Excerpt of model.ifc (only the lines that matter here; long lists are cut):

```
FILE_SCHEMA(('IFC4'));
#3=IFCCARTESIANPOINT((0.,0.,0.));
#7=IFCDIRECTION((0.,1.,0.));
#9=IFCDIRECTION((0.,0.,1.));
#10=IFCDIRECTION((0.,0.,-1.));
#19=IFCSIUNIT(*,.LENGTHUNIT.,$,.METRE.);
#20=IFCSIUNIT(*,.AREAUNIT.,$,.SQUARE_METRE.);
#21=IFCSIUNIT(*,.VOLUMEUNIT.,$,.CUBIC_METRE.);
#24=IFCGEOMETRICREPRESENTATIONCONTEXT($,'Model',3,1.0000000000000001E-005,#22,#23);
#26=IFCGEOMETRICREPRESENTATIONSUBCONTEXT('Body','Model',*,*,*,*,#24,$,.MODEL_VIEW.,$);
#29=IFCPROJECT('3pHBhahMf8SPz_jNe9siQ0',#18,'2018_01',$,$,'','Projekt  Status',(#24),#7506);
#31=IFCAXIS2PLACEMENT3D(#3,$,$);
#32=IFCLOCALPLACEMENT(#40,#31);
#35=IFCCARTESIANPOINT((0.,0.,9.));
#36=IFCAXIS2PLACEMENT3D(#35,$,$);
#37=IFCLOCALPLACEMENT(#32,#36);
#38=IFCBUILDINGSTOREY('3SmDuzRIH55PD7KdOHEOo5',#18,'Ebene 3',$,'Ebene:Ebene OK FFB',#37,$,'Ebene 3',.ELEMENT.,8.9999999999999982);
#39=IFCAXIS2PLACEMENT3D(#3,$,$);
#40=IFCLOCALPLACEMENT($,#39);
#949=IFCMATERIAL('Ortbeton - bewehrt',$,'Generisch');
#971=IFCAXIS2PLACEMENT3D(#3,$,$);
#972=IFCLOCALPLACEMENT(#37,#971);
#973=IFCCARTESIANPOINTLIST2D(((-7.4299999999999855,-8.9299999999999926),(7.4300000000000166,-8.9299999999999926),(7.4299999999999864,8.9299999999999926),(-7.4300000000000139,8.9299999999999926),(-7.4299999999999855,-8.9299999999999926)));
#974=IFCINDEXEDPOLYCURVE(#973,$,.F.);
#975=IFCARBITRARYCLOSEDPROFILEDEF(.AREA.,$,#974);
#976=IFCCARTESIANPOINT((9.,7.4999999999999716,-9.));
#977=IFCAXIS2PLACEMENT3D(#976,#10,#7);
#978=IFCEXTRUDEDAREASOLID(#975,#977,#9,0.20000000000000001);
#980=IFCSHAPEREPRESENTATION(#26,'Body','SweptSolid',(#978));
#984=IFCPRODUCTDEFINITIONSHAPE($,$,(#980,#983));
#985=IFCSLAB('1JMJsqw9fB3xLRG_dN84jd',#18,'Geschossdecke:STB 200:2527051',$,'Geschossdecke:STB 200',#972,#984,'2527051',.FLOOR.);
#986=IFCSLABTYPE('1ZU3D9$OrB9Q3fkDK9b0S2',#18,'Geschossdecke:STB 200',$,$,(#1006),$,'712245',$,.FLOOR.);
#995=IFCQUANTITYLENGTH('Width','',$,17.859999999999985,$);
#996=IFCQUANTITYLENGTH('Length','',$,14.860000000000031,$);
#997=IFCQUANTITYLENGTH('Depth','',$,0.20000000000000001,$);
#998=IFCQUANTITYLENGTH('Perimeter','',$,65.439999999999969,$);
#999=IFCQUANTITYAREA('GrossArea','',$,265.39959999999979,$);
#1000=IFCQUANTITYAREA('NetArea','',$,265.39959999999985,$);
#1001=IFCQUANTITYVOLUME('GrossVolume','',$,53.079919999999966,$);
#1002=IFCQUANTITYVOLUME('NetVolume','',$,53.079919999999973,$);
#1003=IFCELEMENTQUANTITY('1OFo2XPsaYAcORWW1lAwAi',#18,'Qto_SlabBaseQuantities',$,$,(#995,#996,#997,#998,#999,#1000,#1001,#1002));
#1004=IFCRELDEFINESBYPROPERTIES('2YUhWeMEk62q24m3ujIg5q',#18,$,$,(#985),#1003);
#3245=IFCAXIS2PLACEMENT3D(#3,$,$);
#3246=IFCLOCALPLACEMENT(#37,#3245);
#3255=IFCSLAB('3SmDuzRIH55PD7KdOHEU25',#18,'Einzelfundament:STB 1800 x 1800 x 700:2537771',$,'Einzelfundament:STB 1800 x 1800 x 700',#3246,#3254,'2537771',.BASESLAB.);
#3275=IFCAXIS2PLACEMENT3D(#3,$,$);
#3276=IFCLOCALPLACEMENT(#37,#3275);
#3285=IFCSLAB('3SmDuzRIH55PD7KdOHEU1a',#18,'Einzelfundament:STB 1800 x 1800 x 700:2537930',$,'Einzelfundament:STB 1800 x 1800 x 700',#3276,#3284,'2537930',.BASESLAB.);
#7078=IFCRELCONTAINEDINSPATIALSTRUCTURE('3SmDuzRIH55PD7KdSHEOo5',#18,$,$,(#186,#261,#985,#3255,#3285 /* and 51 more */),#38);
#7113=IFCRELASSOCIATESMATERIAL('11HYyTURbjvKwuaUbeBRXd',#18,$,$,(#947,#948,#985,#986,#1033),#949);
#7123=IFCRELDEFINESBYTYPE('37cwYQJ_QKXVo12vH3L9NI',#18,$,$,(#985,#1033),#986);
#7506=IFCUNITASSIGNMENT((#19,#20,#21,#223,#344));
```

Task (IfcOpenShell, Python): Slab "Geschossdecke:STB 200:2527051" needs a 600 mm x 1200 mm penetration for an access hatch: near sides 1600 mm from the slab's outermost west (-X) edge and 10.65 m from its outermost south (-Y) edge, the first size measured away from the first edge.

```python
import numpy as np
import ifcopenshell
import ifcopenshell.api.feature
import ifcopenshell.api.geometry
import ifcopenshell.api.pset
import ifcopenshell.api.root
import ifcopenshell.geom
import ifcopenshell.util.element
import ifcopenshell.util.placement
import ifcopenshell.util.representation
import ifcopenshell.util.shape
import ifcopenshell.util.unit

model = ifcopenshell.open("model.ifc")
unit_scale = ifcopenshell.util.unit.calculate_unit_scale(model)
area_scale = ifcopenshell.util.unit.calculate_unit_scale(model, "AREAUNIT")
volume_scale = ifcopenshell.util.unit.calculate_unit_scale(model, "VOLUMEUNIT")
settings = ifcopenshell.geom.settings()


def volume(element):
    """Net volume in cubic metres, openings subtracted."""
    shape = ifcopenshell.geom.create_shape(settings, element)
    return ifcopenshell.util.shape.get_volume(shape.geometry)


slab = model.by_guid("1JMJsqw9fB3xLRG_dN84jd")
before = volume(slab)

# Extent in the slab's own axes, in metres. The edges named are its -X and -Y sides.
slab_shape = ifcopenshell.geom.create_shape(settings, slab)
vertices = ifcopenshell.util.shape.get_vertices(slab_shape.geometry)
x_min, y_min, bottom = vertices.min(axis=0)
top = vertices[:, 2].max()

opening = ifcopenshell.api.root.create_entity(model, ifc_class="IfcOpeningElement", name="Access hatch opening", predefined_type="OPENING")
context = ifcopenshell.util.representation.get_context(model, "Model", "Body", "MODEL_VIEW")
width, depth = 0.6, 1.2
outline = [(0.0, 0.0), (width, 0.0), (width, depth), (0.0, depth), (0.0, 0.0)]
# Overshoot both faces by 50 mm so the cut is clean.
shape = ifcopenshell.api.geometry.add_slab_representation(
    model, context=context, depth=top - bottom + 0.1, polyline=outline
)
ifcopenshell.api.geometry.assign_representation(model, product=opening, representation=shape)

matrix = ifcopenshell.util.placement.get_local_placement(slab.ObjectPlacement)
matrix[:, 3] = matrix @ np.append(np.array([x_min + 1.6, y_min + 10.65, bottom - 0.05]) / unit_scale, 1.0)
ifcopenshell.api.geometry.edit_object_placement(model, product=opening, matrix=matrix, is_si=False)
ifcopenshell.api.feature.add_feature(model, feature=opening, element=slab)

after = volume(slab)

# Update the slab's stored quantities.
qto = model.by_id(ifcopenshell.util.element.get_pset(slab, "Qto_SlabBaseQuantities", should_inherit=False)["id"])
ifcopenshell.api.pset.edit_qto(model, qto=qto, properties={
    "NetArea": after / (top - bottom) / area_scale,
    "NetVolume": after / volume_scale,
})

print(f"slab volume {before:.3f} -> {after:.3f} m3")

model.write("model_v2.ifc")
```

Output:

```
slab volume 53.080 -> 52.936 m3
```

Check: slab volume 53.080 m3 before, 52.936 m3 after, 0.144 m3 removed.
